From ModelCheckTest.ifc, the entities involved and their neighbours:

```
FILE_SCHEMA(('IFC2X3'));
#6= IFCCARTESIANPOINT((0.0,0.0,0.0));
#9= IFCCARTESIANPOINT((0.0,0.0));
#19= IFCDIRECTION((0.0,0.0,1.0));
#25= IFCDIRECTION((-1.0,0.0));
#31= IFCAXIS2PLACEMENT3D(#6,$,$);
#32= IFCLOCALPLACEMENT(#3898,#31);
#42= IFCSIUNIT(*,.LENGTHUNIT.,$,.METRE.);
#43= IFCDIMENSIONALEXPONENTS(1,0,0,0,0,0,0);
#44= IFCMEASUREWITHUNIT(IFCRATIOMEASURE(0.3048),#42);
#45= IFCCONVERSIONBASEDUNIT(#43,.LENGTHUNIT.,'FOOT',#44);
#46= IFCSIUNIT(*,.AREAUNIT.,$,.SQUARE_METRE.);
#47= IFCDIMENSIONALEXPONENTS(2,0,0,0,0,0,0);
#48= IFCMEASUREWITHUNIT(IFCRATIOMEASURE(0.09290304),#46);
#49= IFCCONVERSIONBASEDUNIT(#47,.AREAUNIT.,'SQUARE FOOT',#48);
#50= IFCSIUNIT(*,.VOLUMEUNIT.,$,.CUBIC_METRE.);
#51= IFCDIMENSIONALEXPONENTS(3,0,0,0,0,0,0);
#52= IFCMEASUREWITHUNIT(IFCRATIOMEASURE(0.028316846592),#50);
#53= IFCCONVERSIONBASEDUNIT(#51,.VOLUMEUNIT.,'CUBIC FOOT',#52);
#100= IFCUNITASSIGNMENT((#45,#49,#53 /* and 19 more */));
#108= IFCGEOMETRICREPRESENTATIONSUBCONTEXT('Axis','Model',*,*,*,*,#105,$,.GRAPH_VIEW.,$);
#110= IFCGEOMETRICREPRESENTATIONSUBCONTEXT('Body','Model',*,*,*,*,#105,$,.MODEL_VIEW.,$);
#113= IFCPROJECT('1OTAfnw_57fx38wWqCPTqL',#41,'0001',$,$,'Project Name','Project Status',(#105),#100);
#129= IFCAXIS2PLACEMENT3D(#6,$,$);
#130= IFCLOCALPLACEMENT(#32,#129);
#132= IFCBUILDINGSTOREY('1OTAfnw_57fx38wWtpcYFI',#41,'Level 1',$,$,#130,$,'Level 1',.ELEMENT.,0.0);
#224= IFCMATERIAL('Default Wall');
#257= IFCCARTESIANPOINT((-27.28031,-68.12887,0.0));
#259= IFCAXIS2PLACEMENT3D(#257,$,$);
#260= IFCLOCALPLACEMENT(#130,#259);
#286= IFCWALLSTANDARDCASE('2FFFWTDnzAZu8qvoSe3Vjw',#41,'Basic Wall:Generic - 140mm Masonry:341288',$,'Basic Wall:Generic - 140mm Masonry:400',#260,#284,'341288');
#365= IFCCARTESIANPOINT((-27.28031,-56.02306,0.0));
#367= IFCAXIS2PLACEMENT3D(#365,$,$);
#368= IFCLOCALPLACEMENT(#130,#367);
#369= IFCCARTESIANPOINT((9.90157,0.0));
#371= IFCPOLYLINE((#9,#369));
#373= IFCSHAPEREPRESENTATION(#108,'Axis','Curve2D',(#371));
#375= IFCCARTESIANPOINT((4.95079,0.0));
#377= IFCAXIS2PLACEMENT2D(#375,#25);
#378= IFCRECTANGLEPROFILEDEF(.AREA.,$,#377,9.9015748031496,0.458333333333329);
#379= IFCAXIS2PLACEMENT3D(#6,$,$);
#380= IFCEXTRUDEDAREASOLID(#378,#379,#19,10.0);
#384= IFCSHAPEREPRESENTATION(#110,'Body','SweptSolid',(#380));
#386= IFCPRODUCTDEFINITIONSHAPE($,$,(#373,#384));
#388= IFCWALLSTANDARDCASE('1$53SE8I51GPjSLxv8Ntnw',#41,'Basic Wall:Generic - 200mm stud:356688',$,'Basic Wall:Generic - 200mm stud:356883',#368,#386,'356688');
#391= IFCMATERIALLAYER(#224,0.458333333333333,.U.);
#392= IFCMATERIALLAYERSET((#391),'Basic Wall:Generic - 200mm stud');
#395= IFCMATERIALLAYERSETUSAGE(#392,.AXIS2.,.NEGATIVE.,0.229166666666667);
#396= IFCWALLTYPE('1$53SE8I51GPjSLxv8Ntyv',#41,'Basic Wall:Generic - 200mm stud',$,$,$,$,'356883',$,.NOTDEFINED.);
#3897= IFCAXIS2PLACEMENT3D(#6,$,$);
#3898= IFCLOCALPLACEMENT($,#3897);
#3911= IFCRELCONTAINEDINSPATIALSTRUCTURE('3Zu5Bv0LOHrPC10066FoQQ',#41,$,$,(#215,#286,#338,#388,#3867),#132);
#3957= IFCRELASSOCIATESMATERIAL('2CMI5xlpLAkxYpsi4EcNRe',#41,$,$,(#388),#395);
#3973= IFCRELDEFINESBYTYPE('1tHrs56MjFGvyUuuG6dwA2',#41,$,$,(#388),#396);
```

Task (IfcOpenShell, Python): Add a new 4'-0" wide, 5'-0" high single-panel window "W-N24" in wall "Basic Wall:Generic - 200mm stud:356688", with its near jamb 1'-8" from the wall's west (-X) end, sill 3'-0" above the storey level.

```python
import numpy as np
import ifcopenshell
import ifcopenshell.api.feature
import ifcopenshell.api.geometry
import ifcopenshell.api.root
import ifcopenshell.api.spatial
import ifcopenshell.api.type
import ifcopenshell.geom
import ifcopenshell.util.element
import ifcopenshell.util.placement
import ifcopenshell.util.representation
import ifcopenshell.util.shape
import ifcopenshell.util.unit

model = ifcopenshell.open("ModelCheckTest.ifc")
unit_scale = ifcopenshell.util.unit.calculate_unit_scale(model)
settings = ifcopenshell.geom.settings()


def volume(element):
    """Net volume in cubic metres, openings subtracted."""
    shape = ifcopenshell.geom.create_shape(settings, element)
    return ifcopenshell.util.shape.get_volume(shape.geometry)


wall = model.by_guid("1$53SE8I51GPjSLxv8Ntnw")
storey = ifcopenshell.util.element.get_container(wall, ifc_class="IfcBuildingStorey")
context = ifcopenshell.util.representation.get_context(model, "Model", "Body", "MODEL_VIEW")
before = volume(wall)

width, height, from_end, sill = 1.2192, 1.524, 0.508, 0.9144  # metres

# The wall runs along its own X axis, and the end named is its -X end.
wall_shape = ifcopenshell.geom.create_shape(settings, wall)
x, y, z = ifcopenshell.util.shape.get_vertices(wall_shape.geometry).T
start = x.min() + from_end
face, thickness = float(y.min()), float(y.max() - y.min())
wall_matrix = ifcopenshell.util.placement.get_local_placement(wall.ObjectPlacement)
level = ifcopenshell.util.placement.get_local_placement(storey.ObjectPlacement)[2, 3]


def in_wall(x, y):
    """Placement at x, y metres in the wall's axes, at sill height."""
    matrix = wall_matrix.copy()
    matrix[:, 3] = wall_matrix @ np.array([x / unit_scale, y / unit_scale, 0.0, 1.0])
    matrix[2, 3] = level + sill / unit_scale
    return matrix


# Opening: a box that overshoots both wall faces by 50 mm.
opening = ifcopenshell.api.root.create_entity(model, ifc_class="IfcOpeningElement")
box = ifcopenshell.api.geometry.add_wall_representation(
    model, context=context, length=width, height=height, thickness=thickness + 0.1
)
ifcopenshell.api.geometry.assign_representation(model, product=opening, representation=box)
ifcopenshell.api.geometry.edit_object_placement(model, product=opening, matrix=in_wall(start, face - 0.05), is_si=False)
ifcopenshell.api.feature.add_feature(model, feature=opening, element=wall)

window = ifcopenshell.api.root.create_entity(model, ifc_class="IfcWindow", name="W-N24")
window.OverallWidth, window.OverallHeight = width / unit_scale, height / unit_scale
body = ifcopenshell.api.geometry.add_window_representation(
    model,
    context=context,
    overall_width=window.OverallWidth,
    overall_height=window.OverallHeight,
    partition_type="SINGLE_PANEL",
)
ifcopenshell.api.geometry.assign_representation(model, product=window, representation=body)
ifcopenshell.api.spatial.assign_container(model, products=[window], relating_structure=storey)
fills = ifcopenshell.api.feature.add_filling(model, opening=opening, element=window)
fills.OwnerHistory = window.OwnerHistory  # required in IFC2X3

# IFC2X3 keeps the operation on the window style.
style = ifcopenshell.api.root.create_entity(model, ifc_class="IfcWindowStyle", name="W-N24")
style.OperationType, style.ConstructionType = "SINGLE_PANEL", "NOTDEFINED"
style.ParameterTakesPrecedence = style.Sizeable = False
ifcopenshell.api.type.assign_type(model, related_objects=[window], relating_type=style)

# Centre the window in the wall's thickness.
ifcopenshell.api.geometry.edit_object_placement(model, product=window, matrix=in_wall(start, face), is_si=False)
window_shape = ifcopenshell.geom.create_shape(settings, window)
depth = ifcopenshell.util.shape.get_vertices(window_shape.geometry)[:, 1]
offset = face + thickness / 2 - (depth.min() + depth.max()) / 2
ifcopenshell.api.geometry.edit_object_placement(model, product=window, matrix=in_wall(start, offset), is_si=False)

after = volume(wall)

print(f"wall volume {before:.3f} -> {after:.3f} m3")

model.write("ModelCheckTest_edited.ifc")
```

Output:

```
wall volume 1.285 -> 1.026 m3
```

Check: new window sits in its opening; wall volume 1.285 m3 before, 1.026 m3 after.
